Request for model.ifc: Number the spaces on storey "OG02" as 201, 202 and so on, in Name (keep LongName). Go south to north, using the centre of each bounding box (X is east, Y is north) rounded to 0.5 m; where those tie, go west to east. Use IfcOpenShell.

First a look at what the model holds.

```python
import ifcopenshell
import ifcopenshell.util.element
import ifcopenshell.util.placement

model = ifcopenshell.open("model.ifc")
print(model.schema)
storey = next(s for s in model.by_type("IfcBuildingStorey") if s.Name == "OG02")
spaces = [e for e in ifcopenshell.util.element.get_decomposition(storey) if e.is_a("IfcSpace")]
for e in sorted(spaces, key=lambda e: e.id()):
    origin = ifcopenshell.util.placement.get_local_placement(e.ObjectPlacement)[:3, 3]
    print(e.id(), e.Name, e.LongName, origin.round(2) + 0.0, sep=" | ")
```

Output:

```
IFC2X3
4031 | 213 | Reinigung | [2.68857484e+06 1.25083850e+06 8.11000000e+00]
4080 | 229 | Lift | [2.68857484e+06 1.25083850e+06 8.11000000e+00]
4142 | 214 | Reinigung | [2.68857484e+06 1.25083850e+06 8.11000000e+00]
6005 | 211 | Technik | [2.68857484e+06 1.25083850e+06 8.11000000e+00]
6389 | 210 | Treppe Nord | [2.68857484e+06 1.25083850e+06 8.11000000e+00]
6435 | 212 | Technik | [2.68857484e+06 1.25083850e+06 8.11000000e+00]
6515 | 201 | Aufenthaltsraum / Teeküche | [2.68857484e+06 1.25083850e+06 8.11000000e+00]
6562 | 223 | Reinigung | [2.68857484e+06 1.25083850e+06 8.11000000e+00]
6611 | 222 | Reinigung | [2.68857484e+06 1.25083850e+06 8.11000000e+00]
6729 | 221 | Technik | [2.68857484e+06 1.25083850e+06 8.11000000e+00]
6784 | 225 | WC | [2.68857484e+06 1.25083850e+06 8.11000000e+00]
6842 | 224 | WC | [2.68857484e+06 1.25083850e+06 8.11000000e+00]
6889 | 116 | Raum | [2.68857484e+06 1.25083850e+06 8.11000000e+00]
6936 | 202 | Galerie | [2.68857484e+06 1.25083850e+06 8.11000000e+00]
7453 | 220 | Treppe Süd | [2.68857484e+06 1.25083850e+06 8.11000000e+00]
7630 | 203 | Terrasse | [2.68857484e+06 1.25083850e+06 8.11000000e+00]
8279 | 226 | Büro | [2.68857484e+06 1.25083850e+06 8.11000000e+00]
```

```python
import ifcopenshell
import ifcopenshell.geom
import ifcopenshell.util.element
import ifcopenshell.util.shape

model = ifcopenshell.open("model.ifc")
settings = ifcopenshell.geom.settings()
settings.set("use-world-coords", True)


def centre(element):
    shape = ifcopenshell.geom.create_shape(settings, element)
    return ifcopenshell.util.shape.get_bbox_centroid(shape.geometry)


storey = next(s for s in model.by_type("IfcBuildingStorey") if s.Name == "OG02")
spaces = [e for e in ifcopenshell.util.element.get_decomposition(storey) if e.is_a("IfcSpace")]

# Insertion points can sit at a corner or the storey origin, so sort by the geometry (in metres).
centres = {e: centre(e) for e in spaces}
spaces.sort(key=lambda e: (round(centres[e][1] / 0.5), centres[e][0]))

for i, e in enumerate(spaces, start=1):
    number = f"2{i:02d}"
    e.Name = number
    print(e.id(), number)

model.write("model_v2.ifc")
```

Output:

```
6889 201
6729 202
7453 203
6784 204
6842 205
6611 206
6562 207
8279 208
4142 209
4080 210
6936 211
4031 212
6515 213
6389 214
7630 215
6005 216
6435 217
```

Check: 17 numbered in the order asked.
